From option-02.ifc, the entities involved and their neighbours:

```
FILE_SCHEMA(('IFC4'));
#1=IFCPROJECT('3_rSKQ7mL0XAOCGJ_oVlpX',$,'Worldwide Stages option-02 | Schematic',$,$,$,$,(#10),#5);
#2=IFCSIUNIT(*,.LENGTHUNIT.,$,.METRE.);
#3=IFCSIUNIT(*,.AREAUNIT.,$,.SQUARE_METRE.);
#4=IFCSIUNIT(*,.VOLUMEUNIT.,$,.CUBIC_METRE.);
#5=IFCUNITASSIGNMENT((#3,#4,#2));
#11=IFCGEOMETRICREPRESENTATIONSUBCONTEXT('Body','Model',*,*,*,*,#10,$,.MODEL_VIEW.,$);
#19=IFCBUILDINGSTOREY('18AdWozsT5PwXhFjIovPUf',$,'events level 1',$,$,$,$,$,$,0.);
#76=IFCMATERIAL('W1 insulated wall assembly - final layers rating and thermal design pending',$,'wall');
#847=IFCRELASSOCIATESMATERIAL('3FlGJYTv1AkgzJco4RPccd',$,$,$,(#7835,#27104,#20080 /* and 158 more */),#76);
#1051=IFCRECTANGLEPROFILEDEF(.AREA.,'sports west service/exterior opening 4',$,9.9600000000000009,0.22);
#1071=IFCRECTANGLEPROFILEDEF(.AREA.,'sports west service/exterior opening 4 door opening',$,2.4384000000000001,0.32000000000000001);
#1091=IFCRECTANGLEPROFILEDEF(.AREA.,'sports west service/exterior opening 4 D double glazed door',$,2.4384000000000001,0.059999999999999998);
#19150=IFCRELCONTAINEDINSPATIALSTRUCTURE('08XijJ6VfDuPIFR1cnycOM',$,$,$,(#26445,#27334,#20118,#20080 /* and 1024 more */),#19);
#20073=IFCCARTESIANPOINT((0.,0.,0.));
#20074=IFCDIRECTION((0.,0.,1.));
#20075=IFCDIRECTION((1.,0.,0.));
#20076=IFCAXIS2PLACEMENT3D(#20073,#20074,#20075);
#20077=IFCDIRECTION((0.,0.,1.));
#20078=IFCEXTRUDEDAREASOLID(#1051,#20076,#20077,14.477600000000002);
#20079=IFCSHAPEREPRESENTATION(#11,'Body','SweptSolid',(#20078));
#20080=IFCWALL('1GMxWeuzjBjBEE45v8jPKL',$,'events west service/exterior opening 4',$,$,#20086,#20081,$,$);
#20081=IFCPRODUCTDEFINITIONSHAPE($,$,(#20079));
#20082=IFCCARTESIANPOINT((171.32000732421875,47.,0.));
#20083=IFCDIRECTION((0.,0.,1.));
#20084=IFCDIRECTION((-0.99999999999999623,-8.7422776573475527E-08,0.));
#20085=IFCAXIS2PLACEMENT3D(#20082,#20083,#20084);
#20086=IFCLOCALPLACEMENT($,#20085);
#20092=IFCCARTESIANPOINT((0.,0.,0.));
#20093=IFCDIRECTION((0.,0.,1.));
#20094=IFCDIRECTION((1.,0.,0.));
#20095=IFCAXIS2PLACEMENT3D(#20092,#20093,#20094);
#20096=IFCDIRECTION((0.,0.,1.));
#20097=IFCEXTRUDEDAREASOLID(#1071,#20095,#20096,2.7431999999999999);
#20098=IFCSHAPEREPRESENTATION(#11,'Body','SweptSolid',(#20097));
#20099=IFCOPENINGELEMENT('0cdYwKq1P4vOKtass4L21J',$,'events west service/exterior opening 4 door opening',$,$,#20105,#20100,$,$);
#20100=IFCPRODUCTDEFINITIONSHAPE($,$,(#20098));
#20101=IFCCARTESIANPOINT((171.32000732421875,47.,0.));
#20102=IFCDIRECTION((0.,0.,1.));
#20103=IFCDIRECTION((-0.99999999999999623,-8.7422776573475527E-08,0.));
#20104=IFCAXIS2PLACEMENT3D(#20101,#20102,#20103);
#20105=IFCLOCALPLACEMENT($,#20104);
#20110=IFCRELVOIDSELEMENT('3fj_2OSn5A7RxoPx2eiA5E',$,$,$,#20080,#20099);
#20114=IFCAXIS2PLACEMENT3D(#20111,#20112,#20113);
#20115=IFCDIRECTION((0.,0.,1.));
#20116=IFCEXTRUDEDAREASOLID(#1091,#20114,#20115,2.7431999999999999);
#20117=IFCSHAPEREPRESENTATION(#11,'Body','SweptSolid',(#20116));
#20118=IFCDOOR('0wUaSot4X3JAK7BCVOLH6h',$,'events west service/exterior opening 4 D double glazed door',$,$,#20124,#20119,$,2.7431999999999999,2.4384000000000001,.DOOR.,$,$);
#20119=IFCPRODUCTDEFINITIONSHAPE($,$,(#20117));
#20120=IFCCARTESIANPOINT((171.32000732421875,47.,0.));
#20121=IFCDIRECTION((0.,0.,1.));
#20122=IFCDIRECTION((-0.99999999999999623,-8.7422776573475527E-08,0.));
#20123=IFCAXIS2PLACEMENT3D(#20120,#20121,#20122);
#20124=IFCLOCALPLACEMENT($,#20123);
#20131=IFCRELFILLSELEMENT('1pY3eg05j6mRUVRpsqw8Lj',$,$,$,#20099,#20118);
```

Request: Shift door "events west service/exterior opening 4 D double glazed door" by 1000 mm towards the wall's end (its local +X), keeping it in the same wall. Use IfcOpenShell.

```python
import ifcopenshell
import ifcopenshell.api.geometry
import ifcopenshell.util.placement
import ifcopenshell.util.unit

model = ifcopenshell.open("option-02.ifc")
unit_scale = ifcopenshell.util.unit.calculate_unit_scale(model)

door = model.by_id(20118)
opening = door.FillsVoids[0].RelatingOpeningElement
wall = opening.VoidsElements[0].RelatingBuildingElement

wall_matrix = ifcopenshell.util.placement.get_local_placement(wall.ObjectPlacement)
shift = wall_matrix[:3, 0] * 1 / unit_scale
before = ifcopenshell.util.placement.get_local_placement(door.ObjectPlacement)[:3, 3].copy()

# The door is not placed relative to its opening, so move both.
for product in (opening, door):
    matrix = ifcopenshell.util.placement.get_local_placement(product.ObjectPlacement)
    matrix[:3, 3] += shift
    ifcopenshell.api.geometry.edit_object_placement(model, product=product, matrix=matrix, is_si=False)

after = ifcopenshell.util.placement.get_local_placement(door.ObjectPlacement)[:3, 3]
print("door moved by", (after - before).round(3) + 0.0)

model.write("option-02_rev.ifc")
```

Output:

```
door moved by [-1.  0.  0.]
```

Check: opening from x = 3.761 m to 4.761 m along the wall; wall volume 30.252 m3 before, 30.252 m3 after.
